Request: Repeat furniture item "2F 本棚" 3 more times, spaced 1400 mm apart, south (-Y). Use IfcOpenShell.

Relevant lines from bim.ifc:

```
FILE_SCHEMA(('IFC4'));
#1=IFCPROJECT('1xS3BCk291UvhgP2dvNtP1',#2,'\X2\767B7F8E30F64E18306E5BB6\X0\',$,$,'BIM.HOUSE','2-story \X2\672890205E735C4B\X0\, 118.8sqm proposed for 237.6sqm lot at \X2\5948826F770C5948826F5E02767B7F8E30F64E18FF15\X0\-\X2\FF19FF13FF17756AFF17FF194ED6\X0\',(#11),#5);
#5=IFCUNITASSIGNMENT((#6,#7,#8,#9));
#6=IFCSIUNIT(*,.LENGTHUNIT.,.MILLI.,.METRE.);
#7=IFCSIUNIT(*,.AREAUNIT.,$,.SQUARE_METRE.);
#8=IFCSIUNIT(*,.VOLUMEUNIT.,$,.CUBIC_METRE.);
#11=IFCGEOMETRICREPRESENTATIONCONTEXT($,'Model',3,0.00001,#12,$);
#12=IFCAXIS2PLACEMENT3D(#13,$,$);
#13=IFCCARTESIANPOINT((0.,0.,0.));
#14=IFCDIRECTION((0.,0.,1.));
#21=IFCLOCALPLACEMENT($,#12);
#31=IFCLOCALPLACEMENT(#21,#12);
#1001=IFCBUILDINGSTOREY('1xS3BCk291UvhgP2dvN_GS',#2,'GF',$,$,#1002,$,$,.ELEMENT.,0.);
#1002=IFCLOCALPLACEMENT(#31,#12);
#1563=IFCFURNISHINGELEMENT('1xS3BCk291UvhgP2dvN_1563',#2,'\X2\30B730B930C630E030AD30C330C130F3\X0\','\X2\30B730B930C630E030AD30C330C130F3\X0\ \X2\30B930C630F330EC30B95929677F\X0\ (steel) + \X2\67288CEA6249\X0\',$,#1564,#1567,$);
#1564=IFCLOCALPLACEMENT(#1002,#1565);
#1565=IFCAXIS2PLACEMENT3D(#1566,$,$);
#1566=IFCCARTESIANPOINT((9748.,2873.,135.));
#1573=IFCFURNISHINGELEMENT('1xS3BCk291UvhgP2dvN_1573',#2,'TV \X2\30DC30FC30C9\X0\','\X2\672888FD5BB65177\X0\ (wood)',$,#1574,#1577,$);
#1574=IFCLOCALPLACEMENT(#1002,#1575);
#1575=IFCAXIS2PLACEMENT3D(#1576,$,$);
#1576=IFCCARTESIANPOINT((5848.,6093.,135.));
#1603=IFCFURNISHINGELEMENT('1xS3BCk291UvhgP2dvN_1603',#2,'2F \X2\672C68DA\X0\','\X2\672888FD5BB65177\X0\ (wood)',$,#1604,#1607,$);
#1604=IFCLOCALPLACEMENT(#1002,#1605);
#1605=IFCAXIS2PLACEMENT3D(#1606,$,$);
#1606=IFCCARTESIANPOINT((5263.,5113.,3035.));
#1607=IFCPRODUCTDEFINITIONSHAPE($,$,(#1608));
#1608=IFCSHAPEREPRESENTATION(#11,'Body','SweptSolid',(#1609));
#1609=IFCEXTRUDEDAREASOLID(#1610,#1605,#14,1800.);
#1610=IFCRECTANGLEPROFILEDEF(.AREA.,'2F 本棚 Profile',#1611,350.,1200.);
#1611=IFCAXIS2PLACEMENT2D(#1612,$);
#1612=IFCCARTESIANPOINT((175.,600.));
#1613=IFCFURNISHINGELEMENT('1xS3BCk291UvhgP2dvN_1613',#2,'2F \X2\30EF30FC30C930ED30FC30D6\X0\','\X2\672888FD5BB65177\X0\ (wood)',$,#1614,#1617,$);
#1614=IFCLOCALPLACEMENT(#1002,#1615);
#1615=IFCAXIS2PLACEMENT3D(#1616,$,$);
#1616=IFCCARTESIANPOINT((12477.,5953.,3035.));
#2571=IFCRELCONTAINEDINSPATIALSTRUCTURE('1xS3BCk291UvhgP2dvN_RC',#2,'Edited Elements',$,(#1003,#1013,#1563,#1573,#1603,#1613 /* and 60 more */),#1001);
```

```python
import numpy as np
import ifcopenshell
import ifcopenshell.api.geometry
import ifcopenshell.api.root
import ifcopenshell.util.element
import ifcopenshell.util.placement
import ifcopenshell.util.unit

model = ifcopenshell.open("bim.ifc")
unit_scale = ifcopenshell.util.unit.calculate_unit_scale(model)


def reuse_history(source, copy):
    """copy_class also copies each property set's owner history, people and application; keep the originals."""
    for rel in copy.IsDefinedBy:
        if rel.is_a("IfcRelDefinesByProperties") and (history := rel.RelatingPropertyDefinition.OwnerHistory):
            rel.RelatingPropertyDefinition.OwnerHistory = source.OwnerHistory
            ifcopenshell.util.element.remove_deep2(model, history)


source = model.by_guid("1xS3BCk291UvhgP2dvN_1603")
base = ifcopenshell.util.placement.get_local_placement(source.ObjectPlacement)
step = np.array([0.0, -1.0, 0.0]) * 1.4 / unit_scale

for i in range(1, 4):
    copy = ifcopenshell.api.root.copy_class(model, product=source)
    copy.Representation = ifcopenshell.util.element.copy_deep(
        model, source.Representation, exclude=["IfcGeometricRepresentationContext", "IfcRepresentationMap"]
    )
    reuse_history(source, copy)
    matrix = base.copy()
    matrix[:3, 3] += i * step
    print("added at", matrix[:3, 3].round(3) + 0.0)
    ifcopenshell.api.geometry.edit_object_placement(model, product=copy, matrix=matrix, is_si=False)

model.write("bim-out.ifc")
```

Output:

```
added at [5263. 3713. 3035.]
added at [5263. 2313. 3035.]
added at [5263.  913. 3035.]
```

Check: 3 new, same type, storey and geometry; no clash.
